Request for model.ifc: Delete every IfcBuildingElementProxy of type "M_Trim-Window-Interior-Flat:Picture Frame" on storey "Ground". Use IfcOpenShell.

First a look at what the model holds.

```python
import ifcopenshell
import ifcopenshell.util.element

model = ifcopenshell.open("model.ifc")
print(model.schema)
storey = next(s for s in model.by_type("IfcBuildingStorey") if s.Name == "Ground")
proxies = [e for e in ifcopenshell.util.element.get_decomposition(storey) if e.is_a("IfcBuildingElementProxy")]
seen = {}
for e in proxies:
    element_type = ifcopenshell.util.element.get_type(e)
    name = element_type.Name if element_type not in (None, e) else None
    seen[name] = seen.get(name, 0) + 1
for name, count in sorted(seen.items(), key=str):
    print(count, "x", name)
```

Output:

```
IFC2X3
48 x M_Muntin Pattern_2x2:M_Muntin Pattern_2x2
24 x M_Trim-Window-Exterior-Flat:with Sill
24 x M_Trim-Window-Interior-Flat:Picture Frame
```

```python
import ifcopenshell
import ifcopenshell.api.root
import ifcopenshell.util.element

model = ifcopenshell.open("model.ifc")

storey = next(s for s in model.by_type("IfcBuildingStorey") if s.Name == "Ground")
proxies = [e for e in ifcopenshell.util.element.get_decomposition(storey) if e.is_a("IfcBuildingElementProxy")]
targets = [e for e in proxies if (t := ifcopenshell.util.element.get_type(e)) not in (None, e) and t.Name == "M_Trim-Window-Interior-Flat:Picture Frame"]

for e in targets:
    ifcopenshell.api.root.remove_product(model, product=e)
print(len(targets), "removed")

model.write("model_edited.ifc")
```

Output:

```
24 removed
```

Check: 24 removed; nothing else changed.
